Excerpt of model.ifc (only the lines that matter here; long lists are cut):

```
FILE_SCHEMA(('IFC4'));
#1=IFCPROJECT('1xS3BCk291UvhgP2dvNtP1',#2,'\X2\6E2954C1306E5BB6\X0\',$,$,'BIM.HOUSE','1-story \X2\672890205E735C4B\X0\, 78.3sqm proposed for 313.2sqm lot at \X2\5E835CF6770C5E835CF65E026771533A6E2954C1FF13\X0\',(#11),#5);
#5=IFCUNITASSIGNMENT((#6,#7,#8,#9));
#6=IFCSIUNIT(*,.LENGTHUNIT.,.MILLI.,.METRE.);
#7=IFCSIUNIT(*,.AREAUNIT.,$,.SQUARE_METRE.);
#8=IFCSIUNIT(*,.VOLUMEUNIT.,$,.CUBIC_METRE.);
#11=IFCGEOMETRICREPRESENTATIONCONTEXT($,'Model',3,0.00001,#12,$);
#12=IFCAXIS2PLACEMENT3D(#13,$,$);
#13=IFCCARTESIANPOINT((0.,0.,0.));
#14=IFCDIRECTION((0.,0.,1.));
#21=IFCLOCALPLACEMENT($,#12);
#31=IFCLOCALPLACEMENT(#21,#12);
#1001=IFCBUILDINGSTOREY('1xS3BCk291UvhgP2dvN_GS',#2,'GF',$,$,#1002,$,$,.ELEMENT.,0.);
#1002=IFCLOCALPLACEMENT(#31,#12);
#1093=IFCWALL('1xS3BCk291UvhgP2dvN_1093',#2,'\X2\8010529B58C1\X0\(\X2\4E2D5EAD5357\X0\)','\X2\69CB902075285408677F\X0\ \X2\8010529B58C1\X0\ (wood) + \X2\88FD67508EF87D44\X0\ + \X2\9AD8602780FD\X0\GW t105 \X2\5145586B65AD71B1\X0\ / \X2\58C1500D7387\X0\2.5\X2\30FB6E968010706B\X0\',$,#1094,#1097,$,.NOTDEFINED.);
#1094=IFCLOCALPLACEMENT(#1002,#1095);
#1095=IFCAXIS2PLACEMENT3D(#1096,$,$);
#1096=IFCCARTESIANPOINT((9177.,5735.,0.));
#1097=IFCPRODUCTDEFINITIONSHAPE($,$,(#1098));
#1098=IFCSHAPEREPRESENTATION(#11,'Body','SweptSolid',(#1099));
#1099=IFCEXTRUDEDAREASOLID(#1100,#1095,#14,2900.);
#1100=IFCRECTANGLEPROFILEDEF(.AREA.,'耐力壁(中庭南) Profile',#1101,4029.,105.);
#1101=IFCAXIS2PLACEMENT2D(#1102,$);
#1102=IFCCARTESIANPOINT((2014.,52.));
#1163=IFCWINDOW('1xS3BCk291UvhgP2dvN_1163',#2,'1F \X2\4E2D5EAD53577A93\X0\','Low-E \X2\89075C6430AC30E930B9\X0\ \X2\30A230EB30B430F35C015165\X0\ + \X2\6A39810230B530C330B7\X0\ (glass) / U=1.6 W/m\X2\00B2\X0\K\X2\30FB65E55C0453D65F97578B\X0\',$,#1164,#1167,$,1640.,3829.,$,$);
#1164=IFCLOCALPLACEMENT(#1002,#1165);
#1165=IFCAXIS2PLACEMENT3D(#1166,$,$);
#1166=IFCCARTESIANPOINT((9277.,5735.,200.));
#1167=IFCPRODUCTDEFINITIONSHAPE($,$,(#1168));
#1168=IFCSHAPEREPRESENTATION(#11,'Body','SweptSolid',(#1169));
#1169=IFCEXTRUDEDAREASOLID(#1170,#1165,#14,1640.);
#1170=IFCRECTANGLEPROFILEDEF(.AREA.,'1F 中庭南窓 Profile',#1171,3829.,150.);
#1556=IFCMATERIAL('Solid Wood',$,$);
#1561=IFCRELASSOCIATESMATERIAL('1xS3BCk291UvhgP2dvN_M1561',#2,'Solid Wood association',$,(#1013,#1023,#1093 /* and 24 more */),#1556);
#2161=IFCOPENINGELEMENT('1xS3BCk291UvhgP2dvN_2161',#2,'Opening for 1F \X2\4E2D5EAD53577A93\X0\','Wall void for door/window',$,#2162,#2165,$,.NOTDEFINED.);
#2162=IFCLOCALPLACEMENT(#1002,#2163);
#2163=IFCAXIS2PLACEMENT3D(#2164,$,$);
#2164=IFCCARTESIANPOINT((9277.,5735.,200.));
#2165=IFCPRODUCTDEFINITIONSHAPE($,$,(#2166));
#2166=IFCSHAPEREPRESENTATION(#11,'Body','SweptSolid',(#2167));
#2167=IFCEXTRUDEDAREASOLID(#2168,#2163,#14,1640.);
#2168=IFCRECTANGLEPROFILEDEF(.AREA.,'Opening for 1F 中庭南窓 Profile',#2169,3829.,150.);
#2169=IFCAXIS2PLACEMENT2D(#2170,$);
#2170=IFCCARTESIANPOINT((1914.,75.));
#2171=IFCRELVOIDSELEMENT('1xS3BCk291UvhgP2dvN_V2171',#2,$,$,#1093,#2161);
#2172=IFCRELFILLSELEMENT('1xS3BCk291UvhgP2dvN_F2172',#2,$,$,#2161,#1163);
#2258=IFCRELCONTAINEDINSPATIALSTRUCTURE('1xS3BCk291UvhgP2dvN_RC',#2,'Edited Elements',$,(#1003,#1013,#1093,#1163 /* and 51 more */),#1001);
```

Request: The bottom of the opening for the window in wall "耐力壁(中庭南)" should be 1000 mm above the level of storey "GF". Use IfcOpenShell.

```python
import numpy as np
import ifcopenshell
import ifcopenshell.api.geometry
import ifcopenshell.geom
import ifcopenshell.util.element
import ifcopenshell.util.placement
import ifcopenshell.util.shape
import ifcopenshell.util.unit

model = ifcopenshell.open("model.ifc")
unit_scale = ifcopenshell.util.unit.calculate_unit_scale(model)

window = model.by_id(1163)
opening = window.FillsVoids[0].RelatingOpeningElement
storey = ifcopenshell.util.element.get_container(window, ifc_class="IfcBuildingStorey")
level = ifcopenshell.util.placement.get_local_placement(storey.ObjectPlacement)[2, 3]

# The opening's origin need not be at the sill, so measure its lowest point.
shape = ifcopenshell.geom.create_shape(ifcopenshell.geom.settings(), opening)
bottom = ifcopenshell.util.shape.get_shape_bottom_elevation(shape, shape.geometry) / unit_scale
dz = level + 1 / unit_scale - bottom

shift = np.array([0.0, 0.0, dz])
# The window is not placed relative to its opening, so move both.
for product in (opening, window):
    matrix = ifcopenshell.util.placement.get_local_placement(product.ObjectPlacement)
    matrix[:3, 3] += shift
    ifcopenshell.api.geometry.edit_object_placement(model, product=product, matrix=matrix, is_si=False)

print(f"moved by {dz * unit_scale:+.3f} m")

model.write("model_edited.ifc")
```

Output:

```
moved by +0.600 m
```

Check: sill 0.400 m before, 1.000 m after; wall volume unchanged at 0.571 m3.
